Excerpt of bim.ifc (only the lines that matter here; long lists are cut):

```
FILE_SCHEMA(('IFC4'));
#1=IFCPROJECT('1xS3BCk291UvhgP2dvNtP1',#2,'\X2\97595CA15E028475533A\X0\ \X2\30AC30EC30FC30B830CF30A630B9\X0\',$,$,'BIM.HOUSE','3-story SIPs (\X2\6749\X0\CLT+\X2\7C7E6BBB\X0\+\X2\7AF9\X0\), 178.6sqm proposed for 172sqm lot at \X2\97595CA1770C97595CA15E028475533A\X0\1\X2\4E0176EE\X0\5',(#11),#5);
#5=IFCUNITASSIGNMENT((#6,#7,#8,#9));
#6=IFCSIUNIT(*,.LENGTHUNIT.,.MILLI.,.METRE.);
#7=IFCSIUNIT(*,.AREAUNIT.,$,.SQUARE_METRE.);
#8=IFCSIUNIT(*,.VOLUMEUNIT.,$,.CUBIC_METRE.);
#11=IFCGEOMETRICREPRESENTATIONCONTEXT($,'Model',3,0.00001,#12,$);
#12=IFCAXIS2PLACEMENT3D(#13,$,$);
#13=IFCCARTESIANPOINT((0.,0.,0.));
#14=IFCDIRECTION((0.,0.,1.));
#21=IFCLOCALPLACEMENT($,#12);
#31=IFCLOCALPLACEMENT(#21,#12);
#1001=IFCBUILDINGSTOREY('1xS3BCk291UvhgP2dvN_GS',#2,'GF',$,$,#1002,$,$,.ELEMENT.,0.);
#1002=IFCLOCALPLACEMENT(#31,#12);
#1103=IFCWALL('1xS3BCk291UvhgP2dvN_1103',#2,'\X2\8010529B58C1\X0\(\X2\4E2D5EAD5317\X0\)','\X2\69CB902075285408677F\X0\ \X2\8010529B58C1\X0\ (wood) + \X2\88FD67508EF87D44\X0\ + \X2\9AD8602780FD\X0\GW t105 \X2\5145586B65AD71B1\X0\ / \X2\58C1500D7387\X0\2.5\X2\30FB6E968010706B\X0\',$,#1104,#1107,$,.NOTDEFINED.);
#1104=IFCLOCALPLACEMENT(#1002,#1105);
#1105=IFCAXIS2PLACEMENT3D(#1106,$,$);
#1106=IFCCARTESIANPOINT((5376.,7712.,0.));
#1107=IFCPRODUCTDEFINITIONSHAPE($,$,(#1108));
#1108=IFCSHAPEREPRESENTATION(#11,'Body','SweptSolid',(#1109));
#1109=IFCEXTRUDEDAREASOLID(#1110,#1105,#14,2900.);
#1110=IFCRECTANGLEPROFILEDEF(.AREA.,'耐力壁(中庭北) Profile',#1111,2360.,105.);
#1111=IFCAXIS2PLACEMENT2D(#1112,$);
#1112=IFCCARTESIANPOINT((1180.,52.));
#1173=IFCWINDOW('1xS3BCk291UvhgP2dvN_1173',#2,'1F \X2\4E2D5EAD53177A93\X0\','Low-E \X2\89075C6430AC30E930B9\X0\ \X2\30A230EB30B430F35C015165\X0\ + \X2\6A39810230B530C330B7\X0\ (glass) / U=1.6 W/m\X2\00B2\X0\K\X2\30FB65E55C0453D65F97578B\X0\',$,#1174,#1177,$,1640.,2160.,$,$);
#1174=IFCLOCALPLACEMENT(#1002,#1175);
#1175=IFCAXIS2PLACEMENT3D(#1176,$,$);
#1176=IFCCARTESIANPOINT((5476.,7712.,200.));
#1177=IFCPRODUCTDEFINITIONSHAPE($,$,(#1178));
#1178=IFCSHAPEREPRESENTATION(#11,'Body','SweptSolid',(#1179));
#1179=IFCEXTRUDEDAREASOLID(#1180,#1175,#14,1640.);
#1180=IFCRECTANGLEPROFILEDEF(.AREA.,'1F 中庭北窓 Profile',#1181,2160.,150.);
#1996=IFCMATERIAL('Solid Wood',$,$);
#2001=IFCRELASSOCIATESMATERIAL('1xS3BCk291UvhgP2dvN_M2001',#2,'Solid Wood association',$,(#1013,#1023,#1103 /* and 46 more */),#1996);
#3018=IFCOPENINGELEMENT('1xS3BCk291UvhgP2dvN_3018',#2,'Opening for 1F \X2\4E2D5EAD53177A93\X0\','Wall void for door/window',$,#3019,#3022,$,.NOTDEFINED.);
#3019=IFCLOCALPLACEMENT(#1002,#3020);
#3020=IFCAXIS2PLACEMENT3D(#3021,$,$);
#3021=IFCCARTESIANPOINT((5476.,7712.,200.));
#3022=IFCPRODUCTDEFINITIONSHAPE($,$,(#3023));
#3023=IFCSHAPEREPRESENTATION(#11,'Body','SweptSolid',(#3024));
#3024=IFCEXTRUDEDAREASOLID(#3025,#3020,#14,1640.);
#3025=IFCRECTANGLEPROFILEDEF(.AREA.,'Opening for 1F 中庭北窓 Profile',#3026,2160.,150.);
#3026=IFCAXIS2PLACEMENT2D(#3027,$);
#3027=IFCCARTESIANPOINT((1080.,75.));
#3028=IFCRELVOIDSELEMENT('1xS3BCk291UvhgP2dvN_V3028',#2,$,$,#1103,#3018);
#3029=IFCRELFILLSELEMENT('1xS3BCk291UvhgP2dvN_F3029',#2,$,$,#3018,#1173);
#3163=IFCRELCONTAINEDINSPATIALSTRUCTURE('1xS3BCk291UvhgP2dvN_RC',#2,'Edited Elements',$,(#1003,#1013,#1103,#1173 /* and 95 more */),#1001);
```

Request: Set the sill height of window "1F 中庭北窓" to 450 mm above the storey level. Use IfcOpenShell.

```python
import numpy as np
import ifcopenshell
import ifcopenshell.api.geometry
import ifcopenshell.geom
import ifcopenshell.util.element
import ifcopenshell.util.placement
import ifcopenshell.util.shape
import ifcopenshell.util.unit

model = ifcopenshell.open("bim.ifc")
unit_scale = ifcopenshell.util.unit.calculate_unit_scale(model)

window = model.by_guid("1xS3BCk291UvhgP2dvN_1173")
opening = window.FillsVoids[0].RelatingOpeningElement
storey = ifcopenshell.util.element.get_container(window, ifc_class="IfcBuildingStorey")
level = ifcopenshell.util.placement.get_local_placement(storey.ObjectPlacement)[2, 3]

# The opening's origin need not be at the sill, so measure its lowest point.
shape = ifcopenshell.geom.create_shape(ifcopenshell.geom.settings(), opening)
bottom = ifcopenshell.util.shape.get_shape_bottom_elevation(shape, shape.geometry) / unit_scale
dz = level + 450.0 - bottom

shift = np.array([0.0, 0.0, dz])
# The window is not placed relative to its opening, so move both.
for product in (opening, window):
    matrix = ifcopenshell.util.placement.get_local_placement(product.ObjectPlacement)
    matrix[:3, 3] += shift
    ifcopenshell.api.geometry.edit_object_placement(model, product=product, matrix=matrix, is_si=False)

print(f"moved by {dz * unit_scale:+.3f} m")

model.write("bim_edited.ifc")
```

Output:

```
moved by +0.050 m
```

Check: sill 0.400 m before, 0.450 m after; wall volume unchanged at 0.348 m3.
